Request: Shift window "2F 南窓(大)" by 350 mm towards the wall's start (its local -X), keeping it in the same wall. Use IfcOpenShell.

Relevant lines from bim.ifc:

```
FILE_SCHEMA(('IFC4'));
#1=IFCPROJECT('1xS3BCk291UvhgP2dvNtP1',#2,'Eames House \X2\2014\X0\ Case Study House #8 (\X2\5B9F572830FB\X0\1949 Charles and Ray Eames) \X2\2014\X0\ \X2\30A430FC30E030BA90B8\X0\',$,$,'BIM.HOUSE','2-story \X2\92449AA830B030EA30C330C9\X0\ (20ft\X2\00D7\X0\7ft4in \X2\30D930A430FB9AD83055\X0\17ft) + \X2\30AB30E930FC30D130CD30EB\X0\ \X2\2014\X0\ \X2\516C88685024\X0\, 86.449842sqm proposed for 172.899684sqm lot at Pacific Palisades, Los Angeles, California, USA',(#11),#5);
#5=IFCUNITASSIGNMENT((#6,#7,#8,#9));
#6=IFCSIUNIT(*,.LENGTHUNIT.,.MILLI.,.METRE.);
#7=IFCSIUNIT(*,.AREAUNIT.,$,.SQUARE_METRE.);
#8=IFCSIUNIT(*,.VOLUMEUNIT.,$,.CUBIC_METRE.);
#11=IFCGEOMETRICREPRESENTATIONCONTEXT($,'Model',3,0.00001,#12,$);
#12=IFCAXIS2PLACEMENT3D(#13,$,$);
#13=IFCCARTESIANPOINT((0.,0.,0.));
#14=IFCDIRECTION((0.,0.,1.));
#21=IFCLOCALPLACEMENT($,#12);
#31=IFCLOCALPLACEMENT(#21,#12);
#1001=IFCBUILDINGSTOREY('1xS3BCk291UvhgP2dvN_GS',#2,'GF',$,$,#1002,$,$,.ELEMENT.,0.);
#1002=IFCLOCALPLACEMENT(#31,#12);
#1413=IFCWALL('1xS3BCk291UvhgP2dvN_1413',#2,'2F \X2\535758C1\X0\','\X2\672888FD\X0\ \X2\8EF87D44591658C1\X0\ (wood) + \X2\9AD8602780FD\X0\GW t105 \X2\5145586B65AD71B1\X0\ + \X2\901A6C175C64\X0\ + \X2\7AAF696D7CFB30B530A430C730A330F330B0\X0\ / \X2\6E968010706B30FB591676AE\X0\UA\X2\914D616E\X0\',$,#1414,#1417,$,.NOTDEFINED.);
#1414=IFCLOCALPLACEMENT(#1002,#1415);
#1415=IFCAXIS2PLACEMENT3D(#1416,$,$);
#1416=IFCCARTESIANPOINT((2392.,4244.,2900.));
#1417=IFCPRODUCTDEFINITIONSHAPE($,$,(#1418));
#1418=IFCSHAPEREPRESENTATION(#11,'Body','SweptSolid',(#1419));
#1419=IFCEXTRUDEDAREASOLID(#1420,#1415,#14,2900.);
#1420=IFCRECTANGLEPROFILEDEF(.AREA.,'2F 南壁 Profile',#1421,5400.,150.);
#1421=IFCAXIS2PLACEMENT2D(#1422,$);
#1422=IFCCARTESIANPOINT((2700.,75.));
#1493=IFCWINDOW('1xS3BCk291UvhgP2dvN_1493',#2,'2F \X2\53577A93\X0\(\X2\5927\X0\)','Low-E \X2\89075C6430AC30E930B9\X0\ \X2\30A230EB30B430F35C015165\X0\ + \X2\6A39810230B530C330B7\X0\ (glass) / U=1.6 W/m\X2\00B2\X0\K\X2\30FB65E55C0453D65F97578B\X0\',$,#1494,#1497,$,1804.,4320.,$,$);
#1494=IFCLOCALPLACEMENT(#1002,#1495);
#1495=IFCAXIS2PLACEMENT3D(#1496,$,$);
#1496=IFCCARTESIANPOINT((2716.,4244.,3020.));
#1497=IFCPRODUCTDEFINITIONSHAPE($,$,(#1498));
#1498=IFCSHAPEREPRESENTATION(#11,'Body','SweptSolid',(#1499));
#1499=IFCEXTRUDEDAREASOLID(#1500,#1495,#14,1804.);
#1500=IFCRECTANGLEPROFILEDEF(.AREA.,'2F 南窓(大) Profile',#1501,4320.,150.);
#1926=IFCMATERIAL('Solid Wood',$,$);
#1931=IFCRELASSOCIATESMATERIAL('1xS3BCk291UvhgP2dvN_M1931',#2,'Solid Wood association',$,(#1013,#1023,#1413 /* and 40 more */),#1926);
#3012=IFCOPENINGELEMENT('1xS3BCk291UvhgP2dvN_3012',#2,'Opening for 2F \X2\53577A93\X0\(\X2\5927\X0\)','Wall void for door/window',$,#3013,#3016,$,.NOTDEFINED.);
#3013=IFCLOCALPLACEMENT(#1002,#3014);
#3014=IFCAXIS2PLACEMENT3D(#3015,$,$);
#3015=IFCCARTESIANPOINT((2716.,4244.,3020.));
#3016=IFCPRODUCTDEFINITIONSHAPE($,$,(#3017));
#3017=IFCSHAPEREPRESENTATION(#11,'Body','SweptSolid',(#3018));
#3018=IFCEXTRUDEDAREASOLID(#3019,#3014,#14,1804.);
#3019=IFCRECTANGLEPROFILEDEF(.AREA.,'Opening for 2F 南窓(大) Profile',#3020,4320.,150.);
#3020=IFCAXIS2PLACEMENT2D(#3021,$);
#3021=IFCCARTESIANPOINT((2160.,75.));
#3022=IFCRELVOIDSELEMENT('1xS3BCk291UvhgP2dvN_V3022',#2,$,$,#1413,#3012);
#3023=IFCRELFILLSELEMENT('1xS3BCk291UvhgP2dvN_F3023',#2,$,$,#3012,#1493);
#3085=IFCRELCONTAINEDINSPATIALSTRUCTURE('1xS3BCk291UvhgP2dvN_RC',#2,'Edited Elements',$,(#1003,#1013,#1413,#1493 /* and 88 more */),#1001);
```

```python
import ifcopenshell
import ifcopenshell.api.geometry
import ifcopenshell.util.placement
import ifcopenshell.util.unit

model = ifcopenshell.open("bim.ifc")
unit_scale = ifcopenshell.util.unit.calculate_unit_scale(model)

window = model.by_guid("1xS3BCk291UvhgP2dvN_1493")
opening = window.FillsVoids[0].RelatingOpeningElement
wall = opening.VoidsElements[0].RelatingBuildingElement

wall_matrix = ifcopenshell.util.placement.get_local_placement(wall.ObjectPlacement)
shift = wall_matrix[:3, 0] * -0.35 / unit_scale
before = ifcopenshell.util.placement.get_local_placement(window.ObjectPlacement)[:3, 3].copy()

# The window is not placed relative to its opening, so move both.
for product in (opening, window):
    matrix = ifcopenshell.util.placement.get_local_placement(product.ObjectPlacement)
    matrix[:3, 3] += shift
    ifcopenshell.api.geometry.edit_object_placement(model, product=product, matrix=matrix, is_si=False)

after = ifcopenshell.util.placement.get_local_placement(window.ObjectPlacement)[:3, 3]
print("window moved by", (after - before).round(3) + 0.0)

model.write("bim_updated.ifc")
```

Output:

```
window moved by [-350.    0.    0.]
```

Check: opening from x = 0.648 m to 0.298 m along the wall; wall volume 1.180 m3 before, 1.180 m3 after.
